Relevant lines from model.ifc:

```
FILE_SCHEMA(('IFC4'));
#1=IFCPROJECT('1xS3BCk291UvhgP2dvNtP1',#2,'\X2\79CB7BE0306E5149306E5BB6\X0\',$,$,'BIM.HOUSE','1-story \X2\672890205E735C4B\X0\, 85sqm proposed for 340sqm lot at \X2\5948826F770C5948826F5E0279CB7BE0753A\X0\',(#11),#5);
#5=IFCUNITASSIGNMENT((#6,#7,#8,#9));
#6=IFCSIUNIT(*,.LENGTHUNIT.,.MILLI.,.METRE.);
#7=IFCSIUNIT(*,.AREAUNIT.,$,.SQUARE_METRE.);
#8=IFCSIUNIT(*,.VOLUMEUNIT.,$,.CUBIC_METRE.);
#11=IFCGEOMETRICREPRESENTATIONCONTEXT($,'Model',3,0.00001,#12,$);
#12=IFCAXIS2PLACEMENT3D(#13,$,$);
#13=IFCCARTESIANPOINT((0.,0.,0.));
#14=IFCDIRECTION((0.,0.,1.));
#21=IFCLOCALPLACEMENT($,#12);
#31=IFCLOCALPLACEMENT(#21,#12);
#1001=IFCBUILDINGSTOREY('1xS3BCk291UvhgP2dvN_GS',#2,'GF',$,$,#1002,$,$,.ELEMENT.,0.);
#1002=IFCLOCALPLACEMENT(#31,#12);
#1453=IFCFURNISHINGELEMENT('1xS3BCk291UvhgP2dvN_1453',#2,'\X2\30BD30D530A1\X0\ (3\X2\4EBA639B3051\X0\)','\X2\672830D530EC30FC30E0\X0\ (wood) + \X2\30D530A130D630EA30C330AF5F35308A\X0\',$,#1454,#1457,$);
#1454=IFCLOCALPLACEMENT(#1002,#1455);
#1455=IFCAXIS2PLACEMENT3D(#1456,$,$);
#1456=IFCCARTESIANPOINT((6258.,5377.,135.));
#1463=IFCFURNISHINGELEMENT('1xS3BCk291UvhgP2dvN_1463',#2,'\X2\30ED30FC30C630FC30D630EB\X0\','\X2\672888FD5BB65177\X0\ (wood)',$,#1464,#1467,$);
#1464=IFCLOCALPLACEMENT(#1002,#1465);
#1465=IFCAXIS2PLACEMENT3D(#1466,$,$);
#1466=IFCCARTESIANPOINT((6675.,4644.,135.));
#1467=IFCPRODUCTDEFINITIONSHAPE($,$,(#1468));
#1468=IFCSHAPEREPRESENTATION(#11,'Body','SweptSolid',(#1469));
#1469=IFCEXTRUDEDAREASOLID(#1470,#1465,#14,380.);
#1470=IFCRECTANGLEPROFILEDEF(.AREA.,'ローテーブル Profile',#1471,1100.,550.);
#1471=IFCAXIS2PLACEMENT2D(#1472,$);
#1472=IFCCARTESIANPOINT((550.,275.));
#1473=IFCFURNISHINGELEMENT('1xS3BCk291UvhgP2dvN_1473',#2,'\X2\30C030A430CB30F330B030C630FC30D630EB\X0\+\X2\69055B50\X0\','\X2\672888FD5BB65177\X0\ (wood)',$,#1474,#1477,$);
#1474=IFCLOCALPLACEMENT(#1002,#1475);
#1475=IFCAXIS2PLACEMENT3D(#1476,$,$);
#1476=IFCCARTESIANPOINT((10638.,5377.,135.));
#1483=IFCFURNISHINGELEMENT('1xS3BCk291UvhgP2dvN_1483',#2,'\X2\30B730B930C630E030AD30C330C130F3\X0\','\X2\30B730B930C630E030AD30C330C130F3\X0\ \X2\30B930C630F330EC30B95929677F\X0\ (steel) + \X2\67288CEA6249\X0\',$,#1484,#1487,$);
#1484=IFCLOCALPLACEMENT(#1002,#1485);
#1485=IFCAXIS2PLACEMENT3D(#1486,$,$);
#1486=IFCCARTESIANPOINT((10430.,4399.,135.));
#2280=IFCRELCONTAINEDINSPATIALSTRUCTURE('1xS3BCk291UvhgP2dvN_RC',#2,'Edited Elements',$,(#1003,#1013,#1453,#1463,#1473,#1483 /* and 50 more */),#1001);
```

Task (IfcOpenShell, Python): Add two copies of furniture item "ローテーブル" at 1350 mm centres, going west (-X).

```python
import numpy as np
import ifcopenshell
import ifcopenshell.api.geometry
import ifcopenshell.api.root
import ifcopenshell.util.element
import ifcopenshell.util.placement
import ifcopenshell.util.unit

model = ifcopenshell.open("model.ifc")
unit_scale = ifcopenshell.util.unit.calculate_unit_scale(model)


def reuse_history(source, copy):
    """copy_class also copies each property set's owner history, people and application; keep the originals."""
    for rel in copy.IsDefinedBy:
        if rel.is_a("IfcRelDefinesByProperties") and (history := rel.RelatingPropertyDefinition.OwnerHistory):
            rel.RelatingPropertyDefinition.OwnerHistory = source.OwnerHistory
            ifcopenshell.util.element.remove_deep2(model, history)


source = model.by_guid("1xS3BCk291UvhgP2dvN_1463")
base = ifcopenshell.util.placement.get_local_placement(source.ObjectPlacement)
step = np.array([-1.0, 0.0, 0.0]) * 1.35 / unit_scale

for i in range(1, 3):
    copy = ifcopenshell.api.root.copy_class(model, product=source)
    copy.Representation = ifcopenshell.util.element.copy_deep(
        model, source.Representation, exclude=["IfcGeometricRepresentationContext", "IfcRepresentationMap"]
    )
    reuse_history(source, copy)
    matrix = base.copy()
    matrix[:3, 3] += i * step
    print("added at", matrix[:3, 3].round(3) + 0.0)
    ifcopenshell.api.geometry.edit_object_placement(model, product=copy, matrix=matrix, is_si=False)

model.write("model_v2.ifc")
```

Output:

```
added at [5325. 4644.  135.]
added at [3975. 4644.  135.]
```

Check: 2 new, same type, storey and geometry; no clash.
